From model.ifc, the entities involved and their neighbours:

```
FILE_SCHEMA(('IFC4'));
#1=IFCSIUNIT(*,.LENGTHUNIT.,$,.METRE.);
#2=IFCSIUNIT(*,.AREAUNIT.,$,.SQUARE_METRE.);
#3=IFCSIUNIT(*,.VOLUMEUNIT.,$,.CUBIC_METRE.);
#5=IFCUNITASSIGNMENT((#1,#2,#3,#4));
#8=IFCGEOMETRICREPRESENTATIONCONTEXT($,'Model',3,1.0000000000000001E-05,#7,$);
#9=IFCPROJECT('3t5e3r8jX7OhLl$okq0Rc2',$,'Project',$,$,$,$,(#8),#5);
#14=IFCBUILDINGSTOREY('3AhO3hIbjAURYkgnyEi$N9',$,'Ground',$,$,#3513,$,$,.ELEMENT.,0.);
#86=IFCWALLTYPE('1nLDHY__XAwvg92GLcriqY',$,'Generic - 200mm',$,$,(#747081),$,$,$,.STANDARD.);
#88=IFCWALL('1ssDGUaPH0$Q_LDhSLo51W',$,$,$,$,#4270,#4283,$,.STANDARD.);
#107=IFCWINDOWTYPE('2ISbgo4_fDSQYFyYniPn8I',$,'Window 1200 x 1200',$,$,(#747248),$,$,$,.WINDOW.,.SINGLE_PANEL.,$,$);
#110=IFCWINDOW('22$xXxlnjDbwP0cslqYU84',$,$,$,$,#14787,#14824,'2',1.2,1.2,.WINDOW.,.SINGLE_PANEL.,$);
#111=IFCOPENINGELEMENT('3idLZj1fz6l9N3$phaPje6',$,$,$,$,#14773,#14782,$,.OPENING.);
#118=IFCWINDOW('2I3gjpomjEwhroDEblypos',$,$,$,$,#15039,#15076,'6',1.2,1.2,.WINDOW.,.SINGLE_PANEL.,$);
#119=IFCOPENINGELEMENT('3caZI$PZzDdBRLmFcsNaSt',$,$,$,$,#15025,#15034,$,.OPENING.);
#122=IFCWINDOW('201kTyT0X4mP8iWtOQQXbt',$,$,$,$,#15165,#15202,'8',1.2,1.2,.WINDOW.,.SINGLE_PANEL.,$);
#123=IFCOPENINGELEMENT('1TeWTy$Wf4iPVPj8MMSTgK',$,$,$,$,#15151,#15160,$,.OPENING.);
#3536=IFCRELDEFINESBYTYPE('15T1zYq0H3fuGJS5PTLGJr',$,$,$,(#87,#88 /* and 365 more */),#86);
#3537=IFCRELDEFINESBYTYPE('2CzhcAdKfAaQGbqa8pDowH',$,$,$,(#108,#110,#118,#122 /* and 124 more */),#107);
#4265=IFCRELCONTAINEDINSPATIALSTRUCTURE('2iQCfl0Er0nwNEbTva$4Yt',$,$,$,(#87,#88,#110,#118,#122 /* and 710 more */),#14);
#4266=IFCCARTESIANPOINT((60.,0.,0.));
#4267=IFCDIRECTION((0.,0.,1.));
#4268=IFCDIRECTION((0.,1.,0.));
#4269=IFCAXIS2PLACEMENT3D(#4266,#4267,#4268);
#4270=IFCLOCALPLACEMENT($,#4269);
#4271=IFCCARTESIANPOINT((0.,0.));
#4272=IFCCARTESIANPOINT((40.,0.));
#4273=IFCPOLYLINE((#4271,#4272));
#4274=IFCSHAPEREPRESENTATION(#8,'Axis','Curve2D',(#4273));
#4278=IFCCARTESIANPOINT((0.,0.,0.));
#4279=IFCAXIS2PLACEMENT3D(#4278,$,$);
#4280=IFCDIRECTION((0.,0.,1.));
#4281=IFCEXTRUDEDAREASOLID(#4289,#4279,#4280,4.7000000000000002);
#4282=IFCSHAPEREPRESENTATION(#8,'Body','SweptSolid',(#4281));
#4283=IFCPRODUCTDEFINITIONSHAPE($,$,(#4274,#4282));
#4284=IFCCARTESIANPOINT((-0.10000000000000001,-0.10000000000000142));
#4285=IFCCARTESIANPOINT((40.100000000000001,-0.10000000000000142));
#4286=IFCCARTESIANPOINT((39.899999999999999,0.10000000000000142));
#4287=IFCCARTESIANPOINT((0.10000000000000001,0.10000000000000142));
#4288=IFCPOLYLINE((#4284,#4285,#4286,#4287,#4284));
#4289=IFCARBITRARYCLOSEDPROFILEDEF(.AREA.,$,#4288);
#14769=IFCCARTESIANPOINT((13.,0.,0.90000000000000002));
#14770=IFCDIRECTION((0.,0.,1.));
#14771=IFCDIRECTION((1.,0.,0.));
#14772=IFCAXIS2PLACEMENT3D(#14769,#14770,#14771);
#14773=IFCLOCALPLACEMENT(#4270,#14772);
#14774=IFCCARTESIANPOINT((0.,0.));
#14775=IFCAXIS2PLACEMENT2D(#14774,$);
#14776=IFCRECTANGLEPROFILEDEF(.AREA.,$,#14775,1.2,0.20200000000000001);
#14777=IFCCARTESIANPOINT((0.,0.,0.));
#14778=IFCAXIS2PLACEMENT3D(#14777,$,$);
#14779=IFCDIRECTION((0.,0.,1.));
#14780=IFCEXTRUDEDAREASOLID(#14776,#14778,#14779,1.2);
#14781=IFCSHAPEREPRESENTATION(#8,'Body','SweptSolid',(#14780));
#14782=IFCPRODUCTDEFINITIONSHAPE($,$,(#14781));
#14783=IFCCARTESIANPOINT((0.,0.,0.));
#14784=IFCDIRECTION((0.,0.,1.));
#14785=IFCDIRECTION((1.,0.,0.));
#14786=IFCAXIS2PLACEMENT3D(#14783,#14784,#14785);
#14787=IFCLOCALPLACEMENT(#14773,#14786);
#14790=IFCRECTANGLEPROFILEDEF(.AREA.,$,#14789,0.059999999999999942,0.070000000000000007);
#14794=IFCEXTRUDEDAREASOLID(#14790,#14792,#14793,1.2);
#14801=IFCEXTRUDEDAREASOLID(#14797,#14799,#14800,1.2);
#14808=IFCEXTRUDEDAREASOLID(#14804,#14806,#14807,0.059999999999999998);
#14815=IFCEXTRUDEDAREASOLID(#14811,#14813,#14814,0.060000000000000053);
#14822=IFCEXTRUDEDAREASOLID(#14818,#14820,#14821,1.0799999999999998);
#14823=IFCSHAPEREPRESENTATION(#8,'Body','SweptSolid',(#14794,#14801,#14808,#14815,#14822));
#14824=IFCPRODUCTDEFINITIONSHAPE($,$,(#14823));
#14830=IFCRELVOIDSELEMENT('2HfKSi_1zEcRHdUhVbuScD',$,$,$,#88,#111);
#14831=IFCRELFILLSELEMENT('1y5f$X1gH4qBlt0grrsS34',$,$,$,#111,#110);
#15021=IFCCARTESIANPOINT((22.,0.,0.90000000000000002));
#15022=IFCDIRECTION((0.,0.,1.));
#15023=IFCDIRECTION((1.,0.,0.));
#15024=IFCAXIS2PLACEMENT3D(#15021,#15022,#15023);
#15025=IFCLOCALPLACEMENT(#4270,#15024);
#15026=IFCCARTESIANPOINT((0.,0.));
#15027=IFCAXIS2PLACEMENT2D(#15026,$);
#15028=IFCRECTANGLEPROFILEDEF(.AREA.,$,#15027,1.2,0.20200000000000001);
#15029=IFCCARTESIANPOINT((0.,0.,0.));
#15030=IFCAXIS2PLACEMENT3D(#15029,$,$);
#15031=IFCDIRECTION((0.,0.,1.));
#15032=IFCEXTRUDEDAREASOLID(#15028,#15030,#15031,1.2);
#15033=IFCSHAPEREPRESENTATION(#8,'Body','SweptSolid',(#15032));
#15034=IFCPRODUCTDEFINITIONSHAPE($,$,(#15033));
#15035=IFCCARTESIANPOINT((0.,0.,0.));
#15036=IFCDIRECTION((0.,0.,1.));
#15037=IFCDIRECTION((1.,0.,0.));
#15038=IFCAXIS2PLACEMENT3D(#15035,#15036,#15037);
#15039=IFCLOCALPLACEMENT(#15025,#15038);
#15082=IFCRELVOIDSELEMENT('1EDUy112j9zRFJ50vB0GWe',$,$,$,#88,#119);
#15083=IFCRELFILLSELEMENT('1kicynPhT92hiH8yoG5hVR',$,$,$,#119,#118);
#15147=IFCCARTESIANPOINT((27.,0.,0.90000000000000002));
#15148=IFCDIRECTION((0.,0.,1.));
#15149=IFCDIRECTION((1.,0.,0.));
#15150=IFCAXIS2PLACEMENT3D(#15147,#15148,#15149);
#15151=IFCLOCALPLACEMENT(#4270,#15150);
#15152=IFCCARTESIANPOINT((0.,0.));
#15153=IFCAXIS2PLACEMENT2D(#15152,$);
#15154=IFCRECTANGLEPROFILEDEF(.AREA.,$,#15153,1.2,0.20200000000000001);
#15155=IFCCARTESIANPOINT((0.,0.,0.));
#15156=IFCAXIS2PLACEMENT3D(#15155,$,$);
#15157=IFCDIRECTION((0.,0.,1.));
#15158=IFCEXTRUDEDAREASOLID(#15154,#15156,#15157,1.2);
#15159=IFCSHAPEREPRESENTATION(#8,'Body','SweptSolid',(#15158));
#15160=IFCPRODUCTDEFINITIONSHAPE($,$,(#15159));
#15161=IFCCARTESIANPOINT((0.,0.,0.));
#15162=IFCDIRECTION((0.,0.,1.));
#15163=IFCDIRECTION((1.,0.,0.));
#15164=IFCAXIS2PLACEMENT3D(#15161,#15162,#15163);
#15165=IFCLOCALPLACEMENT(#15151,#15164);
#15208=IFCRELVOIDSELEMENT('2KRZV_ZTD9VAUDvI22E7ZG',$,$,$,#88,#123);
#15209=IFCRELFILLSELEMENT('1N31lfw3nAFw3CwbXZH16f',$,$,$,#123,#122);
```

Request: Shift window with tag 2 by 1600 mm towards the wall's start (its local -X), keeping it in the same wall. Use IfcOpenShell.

```python
import ifcopenshell
import ifcopenshell.api.geometry
import ifcopenshell.util.placement

model = ifcopenshell.open("model.ifc")

window = model.by_guid("22$xXxlnjDbwP0cslqYU84")
opening = window.FillsVoids[0].RelatingOpeningElement
wall = opening.VoidsElements[0].RelatingBuildingElement

wall_matrix = ifcopenshell.util.placement.get_local_placement(wall.ObjectPlacement)
shift = wall_matrix[:3, 0] * -1.6
before = ifcopenshell.util.placement.get_local_placement(window.ObjectPlacement)[:3, 3].copy()

# The window is placed relative to its opening, so it follows when the opening moves.
matrix = ifcopenshell.util.placement.get_local_placement(opening.ObjectPlacement)
matrix[:3, 3] += shift
ifcopenshell.api.geometry.edit_object_placement(
    model, product=opening, matrix=matrix, is_si=False, should_transform_children=True
)

after = ifcopenshell.util.placement.get_local_placement(window.ObjectPlacement)[:3, 3]
print("window moved by", (after - before).round(3) + 0.0)

model.write("model-out.ifc")
```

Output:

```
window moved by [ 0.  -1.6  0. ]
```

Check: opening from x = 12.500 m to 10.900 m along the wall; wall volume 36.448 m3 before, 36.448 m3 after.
